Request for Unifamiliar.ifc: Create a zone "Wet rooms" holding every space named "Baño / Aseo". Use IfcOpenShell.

First a look at what the model holds.

```python
import ifcopenshell

model = ifcopenshell.open("Unifamiliar.ifc")
print(model.schema)
seen = {}
for space in model.by_type("IfcSpace"):
    seen[space.LongName] = seen.get(space.LongName, 0) + 1
for name, count in sorted(seen.items(), key=str):
    print(count, "x", name)
print("zones:", [z.Name for z in model.by_type("IfcZone")][:20])
```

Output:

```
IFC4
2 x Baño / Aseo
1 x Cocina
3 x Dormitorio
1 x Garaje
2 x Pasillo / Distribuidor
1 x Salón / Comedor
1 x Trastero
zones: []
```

```python
import ifcopenshell
import ifcopenshell.api.group
import ifcopenshell.api.root

model = ifcopenshell.open("Unifamiliar.ifc")

names = {"Baño / Aseo"}
spaces = [s for s in model.by_type("IfcSpace") if s.LongName in names]

zone = ifcopenshell.api.root.create_entity(model, ifc_class="IfcZone", name="Wet rooms")
ifcopenshell.api.group.assign_group(model, products=spaces, group=zone)
print(len(spaces), "spaces in", zone.Name)

model.write("Unifamiliar-out.ifc")
```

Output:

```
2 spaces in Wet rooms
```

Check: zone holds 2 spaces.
